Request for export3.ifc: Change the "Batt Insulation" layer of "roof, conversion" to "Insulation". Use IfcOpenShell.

First a look at what the model holds.

```python
import ifcopenshell
import ifcopenshell.util.element

model = ifcopenshell.open("export3.ifc")
print(model.schema)
for layer_set in model.by_type("IfcMaterialLayerSet"):
    if layer_set.LayerSetName == "roof, conversion":
        for layer in layer_set.MaterialLayers:
            print(layer.id(), layer.Material and layer.Material.Name, layer.LayerThickness, sep=" | ")
        print(len(ifcopenshell.util.element.get_elements_by_material(model, layer_set)), "elements and types use it")
print(sorted(m.Name for m in model.by_type("IfcMaterial") if m.Name)[:60])
```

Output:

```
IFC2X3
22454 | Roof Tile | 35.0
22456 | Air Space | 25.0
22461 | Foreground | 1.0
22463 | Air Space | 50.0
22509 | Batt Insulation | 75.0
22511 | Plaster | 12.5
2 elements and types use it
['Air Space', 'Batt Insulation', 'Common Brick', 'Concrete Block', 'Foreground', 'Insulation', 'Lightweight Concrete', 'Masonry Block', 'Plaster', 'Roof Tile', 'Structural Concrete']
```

```python
import ifcopenshell
import ifcopenshell.api.material

model = ifcopenshell.open("export3.ifc")

layer_set = next(s for s in model.by_type("IfcMaterialLayerSet") if s.LayerSetName == "roof, conversion")
layer = next(l for l in layer_set.MaterialLayers if l.Material and l.Material.Name == "Batt Insulation")
material = next(m for m in model.by_type("IfcMaterial") if m.Name == "Insulation")

# Point this one layer at the other material; renaming the old one would change it everywhere.
ifcopenshell.api.material.edit_layer(model, layer=layer, attributes={}, material=material)

print([l.Material.Name if l.Material else None for l in layer_set.MaterialLayers])

model.write("export3_edited.ifc")
```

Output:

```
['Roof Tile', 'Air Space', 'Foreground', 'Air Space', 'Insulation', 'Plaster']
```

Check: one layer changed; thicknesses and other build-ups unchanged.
